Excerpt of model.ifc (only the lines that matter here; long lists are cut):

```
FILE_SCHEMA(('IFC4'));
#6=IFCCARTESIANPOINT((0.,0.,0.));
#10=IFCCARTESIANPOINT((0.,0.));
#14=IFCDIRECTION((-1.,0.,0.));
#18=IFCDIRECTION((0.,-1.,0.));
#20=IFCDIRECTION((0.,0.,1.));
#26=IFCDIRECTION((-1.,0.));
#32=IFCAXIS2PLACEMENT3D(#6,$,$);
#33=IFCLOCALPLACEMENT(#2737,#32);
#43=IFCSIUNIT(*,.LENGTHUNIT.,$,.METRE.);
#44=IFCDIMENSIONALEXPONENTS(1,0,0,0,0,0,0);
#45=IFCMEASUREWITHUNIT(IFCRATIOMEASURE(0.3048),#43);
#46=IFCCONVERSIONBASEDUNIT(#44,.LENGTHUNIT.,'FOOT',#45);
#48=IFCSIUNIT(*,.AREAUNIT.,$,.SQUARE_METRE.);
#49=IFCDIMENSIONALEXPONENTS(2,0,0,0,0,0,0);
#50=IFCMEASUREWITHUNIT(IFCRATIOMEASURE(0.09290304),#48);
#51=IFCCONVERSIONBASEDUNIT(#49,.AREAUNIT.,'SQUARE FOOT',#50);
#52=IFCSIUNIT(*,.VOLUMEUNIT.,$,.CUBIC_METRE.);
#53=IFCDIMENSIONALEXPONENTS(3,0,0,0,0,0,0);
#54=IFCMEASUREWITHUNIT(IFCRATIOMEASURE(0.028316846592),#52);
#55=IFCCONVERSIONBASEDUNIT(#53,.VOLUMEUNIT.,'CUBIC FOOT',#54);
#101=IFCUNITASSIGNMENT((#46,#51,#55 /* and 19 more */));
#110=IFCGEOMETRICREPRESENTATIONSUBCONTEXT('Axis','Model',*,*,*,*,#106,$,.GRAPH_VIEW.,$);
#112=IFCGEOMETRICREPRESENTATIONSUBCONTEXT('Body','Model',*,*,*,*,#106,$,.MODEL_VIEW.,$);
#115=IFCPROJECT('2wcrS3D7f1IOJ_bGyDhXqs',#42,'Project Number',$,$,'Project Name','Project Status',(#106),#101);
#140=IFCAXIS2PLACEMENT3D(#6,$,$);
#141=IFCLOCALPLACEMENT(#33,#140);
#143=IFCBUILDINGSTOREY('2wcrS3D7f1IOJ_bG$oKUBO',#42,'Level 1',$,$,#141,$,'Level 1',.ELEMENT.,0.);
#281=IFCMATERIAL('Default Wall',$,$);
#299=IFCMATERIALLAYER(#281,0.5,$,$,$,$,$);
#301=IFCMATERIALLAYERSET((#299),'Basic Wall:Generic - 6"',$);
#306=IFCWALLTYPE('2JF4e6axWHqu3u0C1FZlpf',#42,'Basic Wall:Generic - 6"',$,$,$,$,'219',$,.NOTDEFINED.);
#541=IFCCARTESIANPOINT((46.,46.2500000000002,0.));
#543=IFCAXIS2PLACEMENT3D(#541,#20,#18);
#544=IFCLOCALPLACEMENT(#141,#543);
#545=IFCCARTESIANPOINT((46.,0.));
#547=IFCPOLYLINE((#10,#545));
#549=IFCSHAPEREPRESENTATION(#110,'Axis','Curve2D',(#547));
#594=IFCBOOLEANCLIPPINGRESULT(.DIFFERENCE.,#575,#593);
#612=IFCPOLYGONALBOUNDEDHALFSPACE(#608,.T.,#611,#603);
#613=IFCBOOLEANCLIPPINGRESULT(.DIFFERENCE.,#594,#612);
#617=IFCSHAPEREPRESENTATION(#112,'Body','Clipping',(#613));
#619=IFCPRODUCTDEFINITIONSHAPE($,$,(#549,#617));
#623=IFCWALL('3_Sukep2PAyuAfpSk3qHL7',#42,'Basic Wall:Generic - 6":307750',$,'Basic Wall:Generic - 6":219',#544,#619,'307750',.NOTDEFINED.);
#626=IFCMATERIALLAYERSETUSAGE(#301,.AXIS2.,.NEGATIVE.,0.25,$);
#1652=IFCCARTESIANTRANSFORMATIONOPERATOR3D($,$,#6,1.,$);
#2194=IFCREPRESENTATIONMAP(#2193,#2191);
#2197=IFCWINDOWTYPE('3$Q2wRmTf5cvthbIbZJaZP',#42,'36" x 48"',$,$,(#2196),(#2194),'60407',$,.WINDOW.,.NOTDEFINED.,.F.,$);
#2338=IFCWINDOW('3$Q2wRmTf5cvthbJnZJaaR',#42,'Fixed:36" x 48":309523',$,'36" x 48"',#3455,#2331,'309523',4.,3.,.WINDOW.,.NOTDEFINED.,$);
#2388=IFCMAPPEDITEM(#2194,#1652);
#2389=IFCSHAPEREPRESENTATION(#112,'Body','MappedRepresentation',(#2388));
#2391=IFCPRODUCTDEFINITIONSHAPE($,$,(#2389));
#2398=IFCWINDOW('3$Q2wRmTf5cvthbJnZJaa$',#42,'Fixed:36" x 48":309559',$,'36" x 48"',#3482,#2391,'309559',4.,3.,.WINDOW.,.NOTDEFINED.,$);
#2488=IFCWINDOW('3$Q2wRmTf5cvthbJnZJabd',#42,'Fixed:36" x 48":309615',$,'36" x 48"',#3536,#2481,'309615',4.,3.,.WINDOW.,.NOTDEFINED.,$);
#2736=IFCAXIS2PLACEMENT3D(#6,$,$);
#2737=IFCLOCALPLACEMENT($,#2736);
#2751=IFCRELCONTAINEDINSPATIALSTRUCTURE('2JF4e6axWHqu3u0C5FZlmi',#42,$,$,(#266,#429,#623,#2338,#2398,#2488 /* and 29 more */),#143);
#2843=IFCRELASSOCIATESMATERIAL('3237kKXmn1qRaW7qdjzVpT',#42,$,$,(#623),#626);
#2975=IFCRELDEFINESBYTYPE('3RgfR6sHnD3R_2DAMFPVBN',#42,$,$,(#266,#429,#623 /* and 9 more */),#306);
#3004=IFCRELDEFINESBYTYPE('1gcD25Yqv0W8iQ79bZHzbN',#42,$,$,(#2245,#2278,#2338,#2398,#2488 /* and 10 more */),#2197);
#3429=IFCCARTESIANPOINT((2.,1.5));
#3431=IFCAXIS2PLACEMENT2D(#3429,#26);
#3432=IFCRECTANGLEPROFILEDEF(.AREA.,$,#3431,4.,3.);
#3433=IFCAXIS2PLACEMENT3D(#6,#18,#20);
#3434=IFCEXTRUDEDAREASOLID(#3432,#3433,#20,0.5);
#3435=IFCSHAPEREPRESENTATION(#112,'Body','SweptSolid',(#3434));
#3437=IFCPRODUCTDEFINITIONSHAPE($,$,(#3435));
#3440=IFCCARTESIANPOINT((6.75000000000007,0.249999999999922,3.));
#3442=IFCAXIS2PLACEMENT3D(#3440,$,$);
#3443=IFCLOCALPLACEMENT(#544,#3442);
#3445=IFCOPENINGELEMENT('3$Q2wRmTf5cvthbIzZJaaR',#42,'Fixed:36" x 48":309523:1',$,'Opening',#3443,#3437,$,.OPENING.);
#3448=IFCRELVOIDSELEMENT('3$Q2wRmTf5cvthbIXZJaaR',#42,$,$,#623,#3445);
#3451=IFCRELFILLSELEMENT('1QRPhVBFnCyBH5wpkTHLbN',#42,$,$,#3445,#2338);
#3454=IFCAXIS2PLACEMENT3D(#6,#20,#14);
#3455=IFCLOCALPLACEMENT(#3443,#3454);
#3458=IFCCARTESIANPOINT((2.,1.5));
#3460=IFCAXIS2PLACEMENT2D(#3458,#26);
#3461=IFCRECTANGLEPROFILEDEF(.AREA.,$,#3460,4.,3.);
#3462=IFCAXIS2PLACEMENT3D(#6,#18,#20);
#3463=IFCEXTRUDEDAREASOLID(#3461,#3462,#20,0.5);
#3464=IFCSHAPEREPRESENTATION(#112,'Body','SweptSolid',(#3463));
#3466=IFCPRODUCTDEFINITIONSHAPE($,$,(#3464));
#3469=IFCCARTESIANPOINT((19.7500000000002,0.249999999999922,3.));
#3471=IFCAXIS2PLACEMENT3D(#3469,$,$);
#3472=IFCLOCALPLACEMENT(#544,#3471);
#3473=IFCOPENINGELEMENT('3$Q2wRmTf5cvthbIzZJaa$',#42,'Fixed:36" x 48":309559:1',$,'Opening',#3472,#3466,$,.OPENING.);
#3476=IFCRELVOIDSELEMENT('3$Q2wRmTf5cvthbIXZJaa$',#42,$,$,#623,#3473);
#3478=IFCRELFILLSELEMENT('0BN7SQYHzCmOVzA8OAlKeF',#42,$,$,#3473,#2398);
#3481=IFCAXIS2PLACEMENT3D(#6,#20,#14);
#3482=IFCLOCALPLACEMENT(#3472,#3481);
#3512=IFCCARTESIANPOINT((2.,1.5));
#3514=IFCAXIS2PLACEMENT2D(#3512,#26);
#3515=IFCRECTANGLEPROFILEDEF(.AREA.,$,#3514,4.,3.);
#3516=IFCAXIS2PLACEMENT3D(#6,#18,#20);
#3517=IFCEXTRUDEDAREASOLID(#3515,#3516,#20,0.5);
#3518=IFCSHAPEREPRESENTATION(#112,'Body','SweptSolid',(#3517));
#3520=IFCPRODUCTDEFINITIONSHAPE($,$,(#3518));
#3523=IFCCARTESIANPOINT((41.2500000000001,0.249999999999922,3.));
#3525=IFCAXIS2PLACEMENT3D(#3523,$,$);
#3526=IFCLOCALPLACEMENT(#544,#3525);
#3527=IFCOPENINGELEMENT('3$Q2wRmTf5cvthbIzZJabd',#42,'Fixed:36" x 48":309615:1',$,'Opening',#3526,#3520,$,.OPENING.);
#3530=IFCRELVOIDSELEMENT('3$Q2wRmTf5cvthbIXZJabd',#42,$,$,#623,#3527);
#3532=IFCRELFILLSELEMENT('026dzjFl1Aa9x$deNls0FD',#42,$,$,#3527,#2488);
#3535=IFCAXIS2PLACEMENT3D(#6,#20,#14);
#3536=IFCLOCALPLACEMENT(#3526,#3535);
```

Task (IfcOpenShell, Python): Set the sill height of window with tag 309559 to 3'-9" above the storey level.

```python
import numpy as np
import ifcopenshell
import ifcopenshell.api.geometry
import ifcopenshell.geom
import ifcopenshell.util.element
import ifcopenshell.util.placement
import ifcopenshell.util.shape
import ifcopenshell.util.unit

model = ifcopenshell.open("model.ifc")
unit_scale = ifcopenshell.util.unit.calculate_unit_scale(model)

window = model.by_guid("3$Q2wRmTf5cvthbJnZJaa$")
opening = window.FillsVoids[0].RelatingOpeningElement
storey = ifcopenshell.util.element.get_container(window, ifc_class="IfcBuildingStorey")
level = ifcopenshell.util.placement.get_local_placement(storey.ObjectPlacement)[2, 3]

# The opening's origin need not be at the sill, so measure its lowest point.
shape = ifcopenshell.geom.create_shape(ifcopenshell.geom.settings(), opening)
bottom = ifcopenshell.util.shape.get_shape_bottom_elevation(shape, shape.geometry) / unit_scale
dz = level + 45 * 0.0254 / unit_scale - bottom

shift = np.array([0.0, 0.0, dz])
# The window is placed relative to its opening, so it follows when the opening moves.
matrix = ifcopenshell.util.placement.get_local_placement(opening.ObjectPlacement)
matrix[:3, 3] += shift
ifcopenshell.api.geometry.edit_object_placement(
    model, product=opening, matrix=matrix, is_si=False, should_transform_children=True
)

print(f"moved by {dz * unit_scale:+.3f} m")

model.write("model_rev.ifc")
```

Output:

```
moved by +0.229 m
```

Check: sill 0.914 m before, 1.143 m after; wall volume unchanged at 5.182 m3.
